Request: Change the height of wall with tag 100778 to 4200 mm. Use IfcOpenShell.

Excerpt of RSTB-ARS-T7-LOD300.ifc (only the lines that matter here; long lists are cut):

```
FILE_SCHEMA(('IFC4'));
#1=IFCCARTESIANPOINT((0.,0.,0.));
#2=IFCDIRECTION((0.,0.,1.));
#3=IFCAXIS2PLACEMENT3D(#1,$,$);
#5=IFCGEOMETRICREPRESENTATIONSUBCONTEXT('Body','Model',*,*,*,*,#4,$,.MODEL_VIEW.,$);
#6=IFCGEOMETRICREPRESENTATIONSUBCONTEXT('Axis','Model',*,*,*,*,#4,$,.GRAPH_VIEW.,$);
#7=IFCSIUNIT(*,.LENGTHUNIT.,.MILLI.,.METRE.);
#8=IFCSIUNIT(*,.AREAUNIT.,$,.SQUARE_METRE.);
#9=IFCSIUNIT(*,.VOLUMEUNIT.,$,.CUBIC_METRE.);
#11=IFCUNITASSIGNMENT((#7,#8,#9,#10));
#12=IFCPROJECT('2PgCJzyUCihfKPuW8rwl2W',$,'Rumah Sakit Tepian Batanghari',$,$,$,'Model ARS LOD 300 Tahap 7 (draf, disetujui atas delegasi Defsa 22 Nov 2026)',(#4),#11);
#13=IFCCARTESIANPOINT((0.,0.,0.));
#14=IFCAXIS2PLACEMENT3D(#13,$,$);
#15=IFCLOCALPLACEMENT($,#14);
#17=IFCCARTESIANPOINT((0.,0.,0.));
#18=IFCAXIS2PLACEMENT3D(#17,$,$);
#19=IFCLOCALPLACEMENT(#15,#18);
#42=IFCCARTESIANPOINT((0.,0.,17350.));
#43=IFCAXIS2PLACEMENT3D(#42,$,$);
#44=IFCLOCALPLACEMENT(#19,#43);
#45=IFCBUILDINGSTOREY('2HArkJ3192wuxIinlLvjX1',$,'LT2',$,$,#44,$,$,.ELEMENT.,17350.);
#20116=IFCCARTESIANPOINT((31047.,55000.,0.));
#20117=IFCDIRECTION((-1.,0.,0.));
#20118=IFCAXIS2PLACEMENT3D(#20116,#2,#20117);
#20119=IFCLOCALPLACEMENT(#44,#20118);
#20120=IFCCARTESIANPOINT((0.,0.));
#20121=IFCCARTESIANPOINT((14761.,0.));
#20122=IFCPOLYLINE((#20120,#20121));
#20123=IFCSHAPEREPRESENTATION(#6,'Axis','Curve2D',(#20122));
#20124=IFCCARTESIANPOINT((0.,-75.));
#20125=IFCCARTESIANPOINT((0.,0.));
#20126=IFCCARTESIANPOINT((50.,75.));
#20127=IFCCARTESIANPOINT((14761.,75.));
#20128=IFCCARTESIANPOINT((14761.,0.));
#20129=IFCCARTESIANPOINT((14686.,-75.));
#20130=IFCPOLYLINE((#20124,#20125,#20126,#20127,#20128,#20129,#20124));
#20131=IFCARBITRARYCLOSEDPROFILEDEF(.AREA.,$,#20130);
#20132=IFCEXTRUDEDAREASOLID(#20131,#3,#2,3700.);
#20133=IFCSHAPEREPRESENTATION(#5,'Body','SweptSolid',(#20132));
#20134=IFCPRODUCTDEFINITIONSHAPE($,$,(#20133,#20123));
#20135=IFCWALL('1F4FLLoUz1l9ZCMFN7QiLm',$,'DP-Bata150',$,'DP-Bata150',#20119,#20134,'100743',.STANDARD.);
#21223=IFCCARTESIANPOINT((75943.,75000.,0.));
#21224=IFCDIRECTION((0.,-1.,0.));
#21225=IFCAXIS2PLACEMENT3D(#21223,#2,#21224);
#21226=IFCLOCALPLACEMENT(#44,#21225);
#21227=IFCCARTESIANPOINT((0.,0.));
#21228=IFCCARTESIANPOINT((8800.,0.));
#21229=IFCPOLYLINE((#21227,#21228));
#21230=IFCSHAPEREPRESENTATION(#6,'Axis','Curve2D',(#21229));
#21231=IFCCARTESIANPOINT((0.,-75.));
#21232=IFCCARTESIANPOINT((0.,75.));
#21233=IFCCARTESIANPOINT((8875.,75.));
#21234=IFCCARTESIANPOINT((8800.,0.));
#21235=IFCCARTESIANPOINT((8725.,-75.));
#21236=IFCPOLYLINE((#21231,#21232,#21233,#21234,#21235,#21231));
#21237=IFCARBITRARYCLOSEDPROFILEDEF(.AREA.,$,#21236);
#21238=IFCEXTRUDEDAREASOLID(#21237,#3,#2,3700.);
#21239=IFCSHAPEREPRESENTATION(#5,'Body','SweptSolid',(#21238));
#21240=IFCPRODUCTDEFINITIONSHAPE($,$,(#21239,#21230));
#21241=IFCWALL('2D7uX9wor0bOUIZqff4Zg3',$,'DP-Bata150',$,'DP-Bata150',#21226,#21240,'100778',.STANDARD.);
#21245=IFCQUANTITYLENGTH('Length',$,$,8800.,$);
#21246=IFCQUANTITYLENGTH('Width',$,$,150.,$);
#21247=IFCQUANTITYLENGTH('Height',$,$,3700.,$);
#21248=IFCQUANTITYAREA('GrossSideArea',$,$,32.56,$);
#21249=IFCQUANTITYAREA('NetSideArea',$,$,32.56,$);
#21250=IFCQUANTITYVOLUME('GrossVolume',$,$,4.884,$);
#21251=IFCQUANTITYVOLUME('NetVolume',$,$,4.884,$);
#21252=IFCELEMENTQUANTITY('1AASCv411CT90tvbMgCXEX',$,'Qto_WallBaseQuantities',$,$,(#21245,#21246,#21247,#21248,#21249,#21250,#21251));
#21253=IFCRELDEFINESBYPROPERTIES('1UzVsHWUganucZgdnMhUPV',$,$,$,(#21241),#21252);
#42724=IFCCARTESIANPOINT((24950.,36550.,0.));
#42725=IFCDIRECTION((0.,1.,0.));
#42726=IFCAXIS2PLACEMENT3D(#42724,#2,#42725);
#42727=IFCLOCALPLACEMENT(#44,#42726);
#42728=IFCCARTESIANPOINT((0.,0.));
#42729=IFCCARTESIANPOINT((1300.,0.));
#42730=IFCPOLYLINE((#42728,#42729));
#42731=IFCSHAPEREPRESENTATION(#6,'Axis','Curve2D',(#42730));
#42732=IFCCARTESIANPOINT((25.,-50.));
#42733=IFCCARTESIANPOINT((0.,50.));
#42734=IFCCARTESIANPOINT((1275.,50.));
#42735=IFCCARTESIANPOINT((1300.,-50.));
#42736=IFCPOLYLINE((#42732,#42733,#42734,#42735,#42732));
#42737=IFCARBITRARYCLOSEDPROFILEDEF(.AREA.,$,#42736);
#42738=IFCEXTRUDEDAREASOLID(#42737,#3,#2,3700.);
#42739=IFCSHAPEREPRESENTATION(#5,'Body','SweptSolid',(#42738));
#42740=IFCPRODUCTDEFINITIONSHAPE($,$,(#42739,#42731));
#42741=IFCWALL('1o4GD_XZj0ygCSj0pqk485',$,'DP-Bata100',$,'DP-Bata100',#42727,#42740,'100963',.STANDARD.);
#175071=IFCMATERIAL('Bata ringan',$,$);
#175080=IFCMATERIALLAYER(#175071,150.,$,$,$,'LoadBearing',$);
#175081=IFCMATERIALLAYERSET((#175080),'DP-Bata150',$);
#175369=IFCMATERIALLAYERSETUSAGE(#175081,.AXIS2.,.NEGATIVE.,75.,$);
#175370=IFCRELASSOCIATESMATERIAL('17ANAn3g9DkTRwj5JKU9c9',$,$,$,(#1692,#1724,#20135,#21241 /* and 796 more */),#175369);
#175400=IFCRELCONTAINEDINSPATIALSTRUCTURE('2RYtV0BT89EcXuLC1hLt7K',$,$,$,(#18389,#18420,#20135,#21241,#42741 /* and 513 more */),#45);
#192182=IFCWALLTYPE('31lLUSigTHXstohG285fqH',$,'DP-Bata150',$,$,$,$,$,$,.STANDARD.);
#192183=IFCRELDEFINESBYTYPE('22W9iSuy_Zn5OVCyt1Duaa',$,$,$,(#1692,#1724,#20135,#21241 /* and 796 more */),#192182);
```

```python
import ifcopenshell
import ifcopenshell.api.pset
import ifcopenshell.geom
import ifcopenshell.util.element
import ifcopenshell.util.representation
import ifcopenshell.util.shape
import ifcopenshell.util.unit

model = ifcopenshell.open("RSTB-ARS-T7-LOD300.ifc")
unit_scale = ifcopenshell.util.unit.calculate_unit_scale(model)
area_scale = ifcopenshell.util.unit.calculate_unit_scale(model, "AREAUNIT")
volume_scale = ifcopenshell.util.unit.calculate_unit_scale(model, "VOLUMEUNIT")
settings = ifcopenshell.geom.settings()


def volume(element):
    """Net volume in cubic metres, openings subtracted."""
    shape = ifcopenshell.geom.create_shape(settings, element)
    return ifcopenshell.util.shape.get_volume(shape.geometry)


wall = model.by_guid("2D7uX9wor0bOUIZqff4Zg3")
before = volume(wall)

body = ifcopenshell.util.representation.get_representation(wall, "Model", "Body")
solid = body.Items[0]
old_height = solid.Depth
solid.Depth = 4.2 / unit_scale
after = volume(wall)
thickness = 0.15  # wall thickness in metres

# Update the stored height, areas and volumes.
qto = model.by_id(ifcopenshell.util.element.get_pset(wall, "Qto_WallBaseQuantities", should_inherit=False)["id"])
ifcopenshell.api.pset.edit_qto(model, qto=qto, properties={
    "Height": solid.Depth,
    "GrossSideArea": ifcopenshell.util.element.get_pset(wall, "Qto_WallBaseQuantities", "GrossSideArea") * solid.Depth / old_height,
    "NetSideArea": after / thickness / area_scale,
    "GrossVolume": ifcopenshell.util.element.get_pset(wall, "Qto_WallBaseQuantities", "GrossVolume") * solid.Depth / old_height,
    "NetVolume": after / volume_scale,
})

print(f"height {old_height:g} -> {solid.Depth:g}, volume {before:.3f} -> {after:.3f} m3")

model.write("RSTB-ARS-T7-LOD300_updated.ifc")
```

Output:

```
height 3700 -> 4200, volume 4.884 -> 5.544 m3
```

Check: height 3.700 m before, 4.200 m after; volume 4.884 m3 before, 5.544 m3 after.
